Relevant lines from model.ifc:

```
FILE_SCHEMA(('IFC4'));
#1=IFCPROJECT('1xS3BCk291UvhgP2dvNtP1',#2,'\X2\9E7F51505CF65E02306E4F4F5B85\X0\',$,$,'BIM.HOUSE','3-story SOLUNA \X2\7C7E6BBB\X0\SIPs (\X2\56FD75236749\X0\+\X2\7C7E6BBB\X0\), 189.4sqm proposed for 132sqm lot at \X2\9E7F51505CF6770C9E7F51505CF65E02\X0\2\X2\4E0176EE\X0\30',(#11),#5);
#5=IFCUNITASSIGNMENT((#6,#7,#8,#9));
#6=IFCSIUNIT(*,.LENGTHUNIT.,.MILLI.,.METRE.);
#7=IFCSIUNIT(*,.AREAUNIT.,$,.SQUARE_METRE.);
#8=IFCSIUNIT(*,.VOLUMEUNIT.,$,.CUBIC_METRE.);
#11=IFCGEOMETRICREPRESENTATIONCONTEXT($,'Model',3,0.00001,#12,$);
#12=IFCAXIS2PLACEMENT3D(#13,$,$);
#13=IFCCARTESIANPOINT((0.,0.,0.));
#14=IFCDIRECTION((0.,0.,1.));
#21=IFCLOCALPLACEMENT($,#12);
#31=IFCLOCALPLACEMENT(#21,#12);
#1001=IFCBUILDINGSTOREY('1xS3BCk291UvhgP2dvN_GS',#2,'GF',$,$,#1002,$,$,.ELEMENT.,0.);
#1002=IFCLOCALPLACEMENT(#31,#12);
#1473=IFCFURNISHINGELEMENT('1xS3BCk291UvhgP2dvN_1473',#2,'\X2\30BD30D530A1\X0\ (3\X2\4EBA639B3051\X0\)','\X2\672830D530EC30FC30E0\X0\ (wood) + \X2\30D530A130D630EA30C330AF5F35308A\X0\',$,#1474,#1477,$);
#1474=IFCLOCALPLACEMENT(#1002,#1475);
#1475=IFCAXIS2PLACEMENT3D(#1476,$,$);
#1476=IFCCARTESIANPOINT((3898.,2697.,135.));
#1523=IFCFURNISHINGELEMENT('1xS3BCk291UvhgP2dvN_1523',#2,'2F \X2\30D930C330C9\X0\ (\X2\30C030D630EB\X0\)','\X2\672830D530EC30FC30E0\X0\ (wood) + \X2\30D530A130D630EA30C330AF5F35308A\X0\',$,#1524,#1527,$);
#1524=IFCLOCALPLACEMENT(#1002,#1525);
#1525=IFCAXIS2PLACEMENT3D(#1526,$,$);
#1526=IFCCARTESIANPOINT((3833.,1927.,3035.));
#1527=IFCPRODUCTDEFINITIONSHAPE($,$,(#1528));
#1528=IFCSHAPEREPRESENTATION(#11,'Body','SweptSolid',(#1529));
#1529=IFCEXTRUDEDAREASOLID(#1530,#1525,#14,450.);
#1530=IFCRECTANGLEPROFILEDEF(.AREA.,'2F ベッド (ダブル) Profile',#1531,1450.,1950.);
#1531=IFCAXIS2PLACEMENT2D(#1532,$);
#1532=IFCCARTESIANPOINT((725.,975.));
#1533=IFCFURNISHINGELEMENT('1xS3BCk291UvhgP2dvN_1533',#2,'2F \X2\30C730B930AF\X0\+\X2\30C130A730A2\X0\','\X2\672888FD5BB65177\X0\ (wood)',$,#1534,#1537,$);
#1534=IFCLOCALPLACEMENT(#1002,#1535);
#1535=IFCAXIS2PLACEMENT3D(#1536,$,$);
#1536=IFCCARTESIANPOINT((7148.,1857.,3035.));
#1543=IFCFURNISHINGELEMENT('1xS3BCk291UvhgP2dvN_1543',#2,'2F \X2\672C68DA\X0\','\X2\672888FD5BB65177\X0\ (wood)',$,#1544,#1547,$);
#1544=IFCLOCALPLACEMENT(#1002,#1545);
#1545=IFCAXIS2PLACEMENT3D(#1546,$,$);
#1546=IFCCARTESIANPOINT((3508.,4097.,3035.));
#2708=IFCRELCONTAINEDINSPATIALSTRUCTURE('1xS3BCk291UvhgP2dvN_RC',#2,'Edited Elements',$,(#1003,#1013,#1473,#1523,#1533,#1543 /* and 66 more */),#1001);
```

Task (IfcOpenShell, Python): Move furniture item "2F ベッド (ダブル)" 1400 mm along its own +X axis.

```python
import ifcopenshell
import ifcopenshell.api.geometry
import ifcopenshell.util.placement
import ifcopenshell.util.unit

model = ifcopenshell.open("model.ifc")
unit_scale = ifcopenshell.util.unit.calculate_unit_scale(model)

item = model.by_id(1523)
matrix = ifcopenshell.util.placement.get_local_placement(item.ObjectPlacement)
matrix[:3, 3] += matrix[:3, 0] * 1.4 / unit_scale
ifcopenshell.api.geometry.edit_object_placement(model, product=item, matrix=matrix, is_si=False)

print(ifcopenshell.util.placement.get_local_placement(item.ObjectPlacement).round(3) + 0.0)

model.write("model_rev.ifc")
```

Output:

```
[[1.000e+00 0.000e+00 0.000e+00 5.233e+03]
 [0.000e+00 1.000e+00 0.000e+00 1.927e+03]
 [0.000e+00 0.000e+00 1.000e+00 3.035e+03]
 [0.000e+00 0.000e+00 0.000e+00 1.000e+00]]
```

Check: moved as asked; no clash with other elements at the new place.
